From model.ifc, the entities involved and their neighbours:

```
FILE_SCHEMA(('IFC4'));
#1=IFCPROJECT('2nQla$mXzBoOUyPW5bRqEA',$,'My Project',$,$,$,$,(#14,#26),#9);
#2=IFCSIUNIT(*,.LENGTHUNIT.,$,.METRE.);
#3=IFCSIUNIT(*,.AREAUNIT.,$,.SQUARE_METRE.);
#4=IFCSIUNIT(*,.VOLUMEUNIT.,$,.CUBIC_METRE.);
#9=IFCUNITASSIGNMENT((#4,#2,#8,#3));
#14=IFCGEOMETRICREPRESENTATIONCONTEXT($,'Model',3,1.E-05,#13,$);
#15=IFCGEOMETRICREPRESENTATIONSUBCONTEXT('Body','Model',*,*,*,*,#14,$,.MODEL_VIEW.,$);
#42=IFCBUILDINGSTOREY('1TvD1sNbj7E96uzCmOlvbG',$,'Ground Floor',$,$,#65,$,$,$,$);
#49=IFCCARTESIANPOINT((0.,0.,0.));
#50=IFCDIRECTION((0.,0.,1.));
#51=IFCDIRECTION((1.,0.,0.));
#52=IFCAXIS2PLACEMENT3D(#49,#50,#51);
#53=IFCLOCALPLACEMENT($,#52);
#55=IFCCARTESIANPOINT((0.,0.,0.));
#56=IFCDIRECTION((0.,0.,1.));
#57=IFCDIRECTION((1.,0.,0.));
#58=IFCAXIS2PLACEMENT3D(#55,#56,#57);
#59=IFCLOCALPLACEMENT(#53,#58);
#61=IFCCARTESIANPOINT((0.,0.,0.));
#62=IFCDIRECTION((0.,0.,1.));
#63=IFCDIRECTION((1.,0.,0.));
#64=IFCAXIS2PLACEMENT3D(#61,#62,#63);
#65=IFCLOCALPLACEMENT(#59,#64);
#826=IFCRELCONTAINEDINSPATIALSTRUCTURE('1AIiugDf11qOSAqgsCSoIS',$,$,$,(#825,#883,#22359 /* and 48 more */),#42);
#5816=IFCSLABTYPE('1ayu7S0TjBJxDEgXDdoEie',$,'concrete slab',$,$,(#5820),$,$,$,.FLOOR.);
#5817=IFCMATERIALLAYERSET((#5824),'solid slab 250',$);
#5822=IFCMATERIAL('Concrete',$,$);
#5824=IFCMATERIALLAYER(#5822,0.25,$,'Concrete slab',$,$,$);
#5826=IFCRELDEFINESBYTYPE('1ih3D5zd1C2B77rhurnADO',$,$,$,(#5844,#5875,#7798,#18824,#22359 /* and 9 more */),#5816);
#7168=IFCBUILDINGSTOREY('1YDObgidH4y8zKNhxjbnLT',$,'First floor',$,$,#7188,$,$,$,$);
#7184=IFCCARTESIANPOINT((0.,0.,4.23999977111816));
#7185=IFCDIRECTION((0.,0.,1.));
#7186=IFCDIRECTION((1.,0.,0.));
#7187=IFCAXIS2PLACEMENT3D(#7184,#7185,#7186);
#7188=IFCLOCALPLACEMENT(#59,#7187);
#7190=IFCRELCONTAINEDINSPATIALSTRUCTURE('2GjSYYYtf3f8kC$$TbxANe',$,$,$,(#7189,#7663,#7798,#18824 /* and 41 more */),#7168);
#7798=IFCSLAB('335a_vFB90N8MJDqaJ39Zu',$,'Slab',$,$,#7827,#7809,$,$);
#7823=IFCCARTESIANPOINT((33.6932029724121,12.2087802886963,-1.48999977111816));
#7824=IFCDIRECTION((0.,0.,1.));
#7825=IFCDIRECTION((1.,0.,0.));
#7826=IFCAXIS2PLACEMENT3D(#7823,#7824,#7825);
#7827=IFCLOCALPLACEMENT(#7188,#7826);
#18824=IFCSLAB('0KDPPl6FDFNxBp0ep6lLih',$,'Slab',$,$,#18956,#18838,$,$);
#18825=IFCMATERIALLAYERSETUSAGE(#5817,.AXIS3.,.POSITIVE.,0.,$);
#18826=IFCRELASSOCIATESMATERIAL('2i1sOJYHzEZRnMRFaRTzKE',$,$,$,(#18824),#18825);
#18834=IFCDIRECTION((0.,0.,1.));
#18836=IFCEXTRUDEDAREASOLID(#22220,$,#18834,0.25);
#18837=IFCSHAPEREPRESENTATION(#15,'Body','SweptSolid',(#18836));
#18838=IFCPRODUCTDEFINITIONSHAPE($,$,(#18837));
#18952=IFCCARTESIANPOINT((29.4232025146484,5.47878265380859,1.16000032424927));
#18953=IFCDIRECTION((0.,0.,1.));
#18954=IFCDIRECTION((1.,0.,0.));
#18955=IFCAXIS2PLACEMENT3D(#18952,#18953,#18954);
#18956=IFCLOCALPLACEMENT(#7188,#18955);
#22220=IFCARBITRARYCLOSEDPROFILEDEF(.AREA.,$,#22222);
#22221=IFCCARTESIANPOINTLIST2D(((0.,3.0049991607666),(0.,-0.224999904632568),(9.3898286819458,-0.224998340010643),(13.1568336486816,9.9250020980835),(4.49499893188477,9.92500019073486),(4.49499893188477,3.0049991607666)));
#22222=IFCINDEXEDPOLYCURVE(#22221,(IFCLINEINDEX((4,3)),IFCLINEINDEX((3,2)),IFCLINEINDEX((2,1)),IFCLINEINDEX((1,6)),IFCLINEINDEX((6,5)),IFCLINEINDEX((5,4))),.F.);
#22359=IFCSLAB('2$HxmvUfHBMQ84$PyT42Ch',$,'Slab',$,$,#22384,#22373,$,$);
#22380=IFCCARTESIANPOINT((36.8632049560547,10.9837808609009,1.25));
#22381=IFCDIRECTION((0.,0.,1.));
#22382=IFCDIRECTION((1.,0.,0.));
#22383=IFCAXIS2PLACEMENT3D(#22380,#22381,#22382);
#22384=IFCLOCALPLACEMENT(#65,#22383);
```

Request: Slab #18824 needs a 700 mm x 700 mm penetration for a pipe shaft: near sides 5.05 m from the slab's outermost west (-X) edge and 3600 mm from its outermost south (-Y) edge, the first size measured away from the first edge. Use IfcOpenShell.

```python
import numpy as np
import ifcopenshell
import ifcopenshell.api.feature
import ifcopenshell.api.geometry
import ifcopenshell.api.root
import ifcopenshell.geom
import ifcopenshell.util.placement
import ifcopenshell.util.representation
import ifcopenshell.util.shape
import ifcopenshell.util.unit

model = ifcopenshell.open("model.ifc")
unit_scale = ifcopenshell.util.unit.calculate_unit_scale(model)
settings = ifcopenshell.geom.settings()


def volume(element):
    """Net volume in cubic metres, openings subtracted."""
    shape = ifcopenshell.geom.create_shape(settings, element)
    return ifcopenshell.util.shape.get_volume(shape.geometry)


slab = model.by_guid("0KDPPl6FDFNxBp0ep6lLih")
before = volume(slab)

# Extent in the slab's own axes, in metres. The edges named are its -X and -Y sides.
slab_shape = ifcopenshell.geom.create_shape(settings, slab)
vertices = ifcopenshell.util.shape.get_vertices(slab_shape.geometry)
x_min, y_min, bottom = vertices.min(axis=0)
top = vertices[:, 2].max()

opening = ifcopenshell.api.root.create_entity(model, ifc_class="IfcOpeningElement", name="Pipe shaft opening", predefined_type="OPENING")
context = ifcopenshell.util.representation.get_context(model, "Model", "Body", "MODEL_VIEW")
width, depth = 0.7, 0.7
outline = [(0.0, 0.0), (width, 0.0), (width, depth), (0.0, depth), (0.0, 0.0)]
# Overshoot both faces by 50 mm so the cut is clean.
shape = ifcopenshell.api.geometry.add_slab_representation(
    model, context=context, depth=top - bottom + 0.1, polyline=outline
)
ifcopenshell.api.geometry.assign_representation(model, product=opening, representation=shape)

matrix = ifcopenshell.util.placement.get_local_placement(slab.ObjectPlacement)
matrix[:, 3] = matrix @ np.append(np.array([x_min + 5.05, y_min + 3.6, bottom - 0.05]) / unit_scale, 1.0)
ifcopenshell.api.geometry.edit_object_placement(model, product=opening, matrix=matrix, is_si=False)
ifcopenshell.api.feature.add_feature(model, feature=opening, element=slab)

after = volume(slab)

print(f"slab volume {before:.3f} -> {after:.3f} m3")

model.write("model_rev.ifc")
```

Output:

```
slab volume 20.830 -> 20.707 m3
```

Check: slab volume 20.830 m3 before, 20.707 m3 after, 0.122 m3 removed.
